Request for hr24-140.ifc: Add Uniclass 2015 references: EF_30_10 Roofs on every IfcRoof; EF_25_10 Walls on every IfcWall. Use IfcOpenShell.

First a look at what the model holds.

```python
import ifcopenshell

model = ifcopenshell.open("hr24-140.ifc")
print(model.schema)
print("classifications:", [c.Name for c in model.by_type("IfcClassification")])
for ifc_class in ("IfcDoor", "IfcRoof", "IfcStair", "IfcWall", "IfcWindow"):
    print(ifc_class, len(model.by_type(ifc_class)))
```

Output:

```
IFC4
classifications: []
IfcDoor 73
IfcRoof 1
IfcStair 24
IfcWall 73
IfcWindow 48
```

```python
import ifcopenshell
import ifcopenshell.api.classification

model = ifcopenshell.open("hr24-140.ifc")

system = ifcopenshell.api.classification.add_classification(model, classification="Uniclass 2015")

codes = {
    "IfcRoof": ("EF_30_10", "Roofs"),
    "IfcWall": ("EF_25_10", "Walls"),
}
for ifc_class, (code, name) in codes.items():
    products = model.by_type(ifc_class)
    ifcopenshell.api.classification.add_reference(
        model, products=products, classification=system, identification=code, name=name
    )
    print(code, len(products))

model.write("hr24-140-out.ifc")
```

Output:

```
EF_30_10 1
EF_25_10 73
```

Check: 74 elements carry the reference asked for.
